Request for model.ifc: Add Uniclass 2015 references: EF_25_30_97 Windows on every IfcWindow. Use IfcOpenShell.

First a look at what the model holds.

```python
import ifcopenshell

model = ifcopenshell.open("model.ifc")
print(model.schema)
print("classifications:", [c.Name for c in model.by_type("IfcClassification")])
for ifc_class in ("IfcDoor", "IfcRoof", "IfcStair", "IfcWall", "IfcWindow"):
    print(ifc_class, len(model.by_type(ifc_class)))
```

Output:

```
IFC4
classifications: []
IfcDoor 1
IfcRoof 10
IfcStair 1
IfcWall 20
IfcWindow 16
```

```python
import ifcopenshell
import ifcopenshell.api.classification

model = ifcopenshell.open("model.ifc")

system = ifcopenshell.api.classification.add_classification(model, classification="Uniclass 2015")

codes = {
    "IfcWindow": ("EF_25_30_97", "Windows"),
}
for ifc_class, (code, name) in codes.items():
    products = model.by_type(ifc_class)
    ifcopenshell.api.classification.add_reference(
        model, products=products, classification=system, identification=code, name=name
    )
    print(code, len(products))

model.write("model-out.ifc")
```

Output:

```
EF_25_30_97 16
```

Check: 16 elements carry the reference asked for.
